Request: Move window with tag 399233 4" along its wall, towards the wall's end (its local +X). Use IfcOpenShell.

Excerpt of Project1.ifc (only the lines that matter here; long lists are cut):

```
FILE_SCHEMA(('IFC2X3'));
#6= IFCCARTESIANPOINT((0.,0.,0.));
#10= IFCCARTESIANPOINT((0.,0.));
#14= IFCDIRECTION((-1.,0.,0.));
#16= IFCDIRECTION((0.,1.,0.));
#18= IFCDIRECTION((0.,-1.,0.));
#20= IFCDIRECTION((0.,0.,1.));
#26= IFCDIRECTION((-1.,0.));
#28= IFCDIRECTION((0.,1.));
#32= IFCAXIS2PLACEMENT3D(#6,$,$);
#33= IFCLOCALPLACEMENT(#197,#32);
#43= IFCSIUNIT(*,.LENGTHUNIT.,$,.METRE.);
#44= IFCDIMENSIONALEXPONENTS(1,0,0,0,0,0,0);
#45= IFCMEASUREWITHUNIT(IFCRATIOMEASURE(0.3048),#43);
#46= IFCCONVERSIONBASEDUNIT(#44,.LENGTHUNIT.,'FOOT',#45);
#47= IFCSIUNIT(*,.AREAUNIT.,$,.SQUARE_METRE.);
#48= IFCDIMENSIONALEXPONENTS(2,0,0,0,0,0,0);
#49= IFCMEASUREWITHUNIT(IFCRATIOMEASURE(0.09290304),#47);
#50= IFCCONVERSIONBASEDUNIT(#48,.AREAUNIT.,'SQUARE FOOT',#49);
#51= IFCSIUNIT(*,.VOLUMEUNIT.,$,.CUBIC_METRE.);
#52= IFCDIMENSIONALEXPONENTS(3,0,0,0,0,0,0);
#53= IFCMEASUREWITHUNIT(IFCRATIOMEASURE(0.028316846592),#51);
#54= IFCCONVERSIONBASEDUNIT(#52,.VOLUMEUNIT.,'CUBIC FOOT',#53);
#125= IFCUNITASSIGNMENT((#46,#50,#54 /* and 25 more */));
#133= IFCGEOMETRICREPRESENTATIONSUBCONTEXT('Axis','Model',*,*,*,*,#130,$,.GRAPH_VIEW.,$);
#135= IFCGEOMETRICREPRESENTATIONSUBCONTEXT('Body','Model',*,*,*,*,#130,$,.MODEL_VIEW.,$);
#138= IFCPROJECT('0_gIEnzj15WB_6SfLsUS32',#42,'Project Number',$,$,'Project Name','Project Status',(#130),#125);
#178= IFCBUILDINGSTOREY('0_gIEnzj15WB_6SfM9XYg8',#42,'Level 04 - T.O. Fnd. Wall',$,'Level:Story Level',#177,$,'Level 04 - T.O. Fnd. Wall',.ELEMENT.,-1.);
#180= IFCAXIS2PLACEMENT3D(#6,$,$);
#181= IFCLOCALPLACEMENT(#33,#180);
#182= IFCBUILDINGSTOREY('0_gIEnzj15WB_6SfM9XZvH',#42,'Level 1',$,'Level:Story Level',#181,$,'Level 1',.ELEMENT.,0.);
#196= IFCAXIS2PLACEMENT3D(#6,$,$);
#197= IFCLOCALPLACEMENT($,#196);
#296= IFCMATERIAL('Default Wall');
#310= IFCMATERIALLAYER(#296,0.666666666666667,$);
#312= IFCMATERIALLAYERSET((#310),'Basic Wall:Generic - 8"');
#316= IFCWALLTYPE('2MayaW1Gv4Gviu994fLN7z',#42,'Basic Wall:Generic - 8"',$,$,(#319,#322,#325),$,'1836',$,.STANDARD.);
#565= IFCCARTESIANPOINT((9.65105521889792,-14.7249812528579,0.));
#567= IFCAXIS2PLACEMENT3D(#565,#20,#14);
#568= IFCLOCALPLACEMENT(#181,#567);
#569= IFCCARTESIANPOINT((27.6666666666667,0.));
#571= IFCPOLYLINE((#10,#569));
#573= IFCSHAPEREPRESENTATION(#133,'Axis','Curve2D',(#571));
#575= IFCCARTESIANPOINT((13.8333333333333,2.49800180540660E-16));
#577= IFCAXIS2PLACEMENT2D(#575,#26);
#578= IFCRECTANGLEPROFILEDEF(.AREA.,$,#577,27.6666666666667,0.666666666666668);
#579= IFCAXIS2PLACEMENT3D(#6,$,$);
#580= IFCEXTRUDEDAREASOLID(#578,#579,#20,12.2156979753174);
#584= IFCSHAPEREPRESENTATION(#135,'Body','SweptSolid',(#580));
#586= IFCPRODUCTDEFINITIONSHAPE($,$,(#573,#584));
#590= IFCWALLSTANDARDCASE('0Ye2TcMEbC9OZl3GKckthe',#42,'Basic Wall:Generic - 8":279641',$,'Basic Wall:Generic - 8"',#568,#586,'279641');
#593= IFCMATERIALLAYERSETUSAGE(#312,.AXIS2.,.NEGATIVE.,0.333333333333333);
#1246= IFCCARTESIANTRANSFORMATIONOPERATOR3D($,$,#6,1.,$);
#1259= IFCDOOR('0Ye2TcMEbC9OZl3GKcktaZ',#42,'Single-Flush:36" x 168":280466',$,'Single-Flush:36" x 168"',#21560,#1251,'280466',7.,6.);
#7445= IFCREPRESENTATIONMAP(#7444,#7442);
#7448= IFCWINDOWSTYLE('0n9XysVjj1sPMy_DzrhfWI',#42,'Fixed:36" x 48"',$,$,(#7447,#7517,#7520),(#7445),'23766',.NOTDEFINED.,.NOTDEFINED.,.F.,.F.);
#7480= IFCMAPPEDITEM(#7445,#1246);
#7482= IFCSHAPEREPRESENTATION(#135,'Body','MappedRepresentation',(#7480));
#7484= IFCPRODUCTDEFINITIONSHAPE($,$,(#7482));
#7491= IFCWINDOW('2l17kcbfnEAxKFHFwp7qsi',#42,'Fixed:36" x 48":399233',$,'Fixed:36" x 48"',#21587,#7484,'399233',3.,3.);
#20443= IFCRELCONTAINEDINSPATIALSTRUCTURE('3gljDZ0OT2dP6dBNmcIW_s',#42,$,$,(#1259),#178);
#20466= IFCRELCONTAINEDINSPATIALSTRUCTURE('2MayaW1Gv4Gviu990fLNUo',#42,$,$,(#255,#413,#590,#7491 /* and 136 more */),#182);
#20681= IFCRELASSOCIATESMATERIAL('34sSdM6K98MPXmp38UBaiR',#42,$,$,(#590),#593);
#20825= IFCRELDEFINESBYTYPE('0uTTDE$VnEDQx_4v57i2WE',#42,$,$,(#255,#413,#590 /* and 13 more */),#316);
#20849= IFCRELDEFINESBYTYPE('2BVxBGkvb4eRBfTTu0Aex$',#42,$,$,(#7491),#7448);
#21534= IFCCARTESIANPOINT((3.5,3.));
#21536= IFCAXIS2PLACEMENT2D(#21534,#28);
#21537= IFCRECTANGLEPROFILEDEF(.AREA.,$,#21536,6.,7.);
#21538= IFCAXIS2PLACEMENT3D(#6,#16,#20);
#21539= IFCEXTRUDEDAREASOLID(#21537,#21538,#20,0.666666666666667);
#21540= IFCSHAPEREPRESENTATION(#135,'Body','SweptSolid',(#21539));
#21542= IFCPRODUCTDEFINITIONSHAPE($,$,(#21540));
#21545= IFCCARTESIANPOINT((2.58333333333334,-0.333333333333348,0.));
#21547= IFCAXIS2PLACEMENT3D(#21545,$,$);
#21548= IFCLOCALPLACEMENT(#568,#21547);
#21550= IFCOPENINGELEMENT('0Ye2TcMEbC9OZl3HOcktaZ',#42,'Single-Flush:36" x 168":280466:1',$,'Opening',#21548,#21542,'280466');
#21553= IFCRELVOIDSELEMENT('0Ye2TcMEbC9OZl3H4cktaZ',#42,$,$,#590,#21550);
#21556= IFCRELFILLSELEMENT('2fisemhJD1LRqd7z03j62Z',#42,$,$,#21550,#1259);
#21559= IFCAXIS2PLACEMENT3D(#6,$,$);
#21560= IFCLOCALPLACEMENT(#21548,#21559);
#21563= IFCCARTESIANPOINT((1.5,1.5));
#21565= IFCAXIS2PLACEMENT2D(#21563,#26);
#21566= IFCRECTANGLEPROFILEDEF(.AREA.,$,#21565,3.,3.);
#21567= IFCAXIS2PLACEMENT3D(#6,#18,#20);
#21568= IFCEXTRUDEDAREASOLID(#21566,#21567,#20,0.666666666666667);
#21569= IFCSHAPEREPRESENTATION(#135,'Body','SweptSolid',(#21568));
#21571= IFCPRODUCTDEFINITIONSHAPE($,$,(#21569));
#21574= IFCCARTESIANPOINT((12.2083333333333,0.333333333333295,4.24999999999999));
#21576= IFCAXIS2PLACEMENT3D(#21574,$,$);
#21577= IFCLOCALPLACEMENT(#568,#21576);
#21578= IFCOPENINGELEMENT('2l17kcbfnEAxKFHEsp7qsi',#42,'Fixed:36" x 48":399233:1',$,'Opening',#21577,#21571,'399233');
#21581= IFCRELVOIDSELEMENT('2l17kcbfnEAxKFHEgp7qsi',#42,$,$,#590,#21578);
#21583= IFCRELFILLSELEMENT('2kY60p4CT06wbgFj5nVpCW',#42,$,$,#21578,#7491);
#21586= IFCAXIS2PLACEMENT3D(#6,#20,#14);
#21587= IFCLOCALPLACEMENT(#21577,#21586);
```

```python
import ifcopenshell
import ifcopenshell.api.geometry
import ifcopenshell.util.placement
import ifcopenshell.util.unit

model = ifcopenshell.open("Project1.ifc")
unit_scale = ifcopenshell.util.unit.calculate_unit_scale(model)

window = model.by_guid("2l17kcbfnEAxKFHFwp7qsi")
opening = window.FillsVoids[0].RelatingOpeningElement
wall = opening.VoidsElements[0].RelatingBuildingElement

wall_matrix = ifcopenshell.util.placement.get_local_placement(wall.ObjectPlacement)
shift = wall_matrix[:3, 0] * 4 * 0.0254 / unit_scale
before = ifcopenshell.util.placement.get_local_placement(window.ObjectPlacement)[:3, 3].copy()

# The window is placed relative to its opening, so it follows when the opening moves.
matrix = ifcopenshell.util.placement.get_local_placement(opening.ObjectPlacement)
matrix[:3, 3] += shift
ifcopenshell.api.geometry.edit_object_placement(
    model, product=opening, matrix=matrix, is_si=False, should_transform_children=True
)

after = ifcopenshell.util.placement.get_local_placement(window.ObjectPlacement)[:3, 3]
print("window moved by", (after - before).round(3) + 0.0)

model.write("Project1_rev.ifc")
```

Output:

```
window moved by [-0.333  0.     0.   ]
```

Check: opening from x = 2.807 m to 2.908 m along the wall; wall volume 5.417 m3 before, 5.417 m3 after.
